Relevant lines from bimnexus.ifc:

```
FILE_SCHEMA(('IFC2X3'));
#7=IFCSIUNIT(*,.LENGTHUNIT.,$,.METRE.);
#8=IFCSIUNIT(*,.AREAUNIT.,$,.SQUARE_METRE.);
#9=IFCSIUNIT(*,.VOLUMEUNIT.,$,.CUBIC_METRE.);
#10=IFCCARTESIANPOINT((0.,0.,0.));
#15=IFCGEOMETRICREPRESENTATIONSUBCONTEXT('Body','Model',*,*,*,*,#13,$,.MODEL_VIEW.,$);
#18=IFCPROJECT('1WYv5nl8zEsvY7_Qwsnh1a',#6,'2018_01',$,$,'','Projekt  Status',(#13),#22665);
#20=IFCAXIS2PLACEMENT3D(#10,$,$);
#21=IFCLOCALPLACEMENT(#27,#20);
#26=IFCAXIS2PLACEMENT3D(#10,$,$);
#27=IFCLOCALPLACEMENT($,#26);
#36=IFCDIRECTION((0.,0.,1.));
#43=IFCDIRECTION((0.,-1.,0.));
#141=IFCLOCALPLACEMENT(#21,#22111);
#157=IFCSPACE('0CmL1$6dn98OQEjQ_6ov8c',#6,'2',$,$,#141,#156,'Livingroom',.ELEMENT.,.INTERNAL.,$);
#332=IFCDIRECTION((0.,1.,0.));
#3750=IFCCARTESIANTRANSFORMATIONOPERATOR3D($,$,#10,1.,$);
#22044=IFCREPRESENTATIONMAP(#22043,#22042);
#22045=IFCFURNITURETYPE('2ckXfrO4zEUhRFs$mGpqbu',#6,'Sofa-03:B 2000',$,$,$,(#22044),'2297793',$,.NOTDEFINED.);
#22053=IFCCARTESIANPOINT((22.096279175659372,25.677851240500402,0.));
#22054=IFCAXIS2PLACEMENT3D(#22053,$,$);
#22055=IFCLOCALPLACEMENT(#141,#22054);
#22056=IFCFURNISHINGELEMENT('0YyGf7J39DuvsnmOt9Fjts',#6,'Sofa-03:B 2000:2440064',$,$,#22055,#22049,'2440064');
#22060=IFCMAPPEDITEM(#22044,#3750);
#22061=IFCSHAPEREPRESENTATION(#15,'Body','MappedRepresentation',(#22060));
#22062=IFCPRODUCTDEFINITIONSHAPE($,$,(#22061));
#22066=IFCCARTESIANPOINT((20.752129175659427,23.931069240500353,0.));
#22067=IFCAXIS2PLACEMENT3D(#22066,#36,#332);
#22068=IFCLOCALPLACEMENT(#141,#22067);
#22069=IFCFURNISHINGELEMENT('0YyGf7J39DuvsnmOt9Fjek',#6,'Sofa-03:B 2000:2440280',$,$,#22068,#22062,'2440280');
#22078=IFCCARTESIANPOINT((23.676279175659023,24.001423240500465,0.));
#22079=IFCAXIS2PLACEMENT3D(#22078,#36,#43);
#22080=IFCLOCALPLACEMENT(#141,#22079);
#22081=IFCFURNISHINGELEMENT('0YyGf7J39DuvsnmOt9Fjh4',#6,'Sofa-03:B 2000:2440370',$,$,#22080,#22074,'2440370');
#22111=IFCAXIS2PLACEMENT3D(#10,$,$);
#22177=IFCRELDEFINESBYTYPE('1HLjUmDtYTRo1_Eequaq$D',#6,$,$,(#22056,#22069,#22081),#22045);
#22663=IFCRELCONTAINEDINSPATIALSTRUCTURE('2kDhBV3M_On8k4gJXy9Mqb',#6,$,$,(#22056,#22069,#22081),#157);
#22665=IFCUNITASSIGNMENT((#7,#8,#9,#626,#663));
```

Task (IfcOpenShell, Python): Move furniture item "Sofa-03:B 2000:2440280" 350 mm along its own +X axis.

```python
import ifcopenshell
import ifcopenshell.api.geometry
import ifcopenshell.util.placement
import ifcopenshell.util.unit

model = ifcopenshell.open("bimnexus.ifc")
unit_scale = ifcopenshell.util.unit.calculate_unit_scale(model)

item = model.by_id(22069)
matrix = ifcopenshell.util.placement.get_local_placement(item.ObjectPlacement)
matrix[:3, 3] += matrix[:3, 0] * 0.35 / unit_scale
ifcopenshell.api.geometry.edit_object_placement(model, product=item, matrix=matrix, is_si=False)

print(ifcopenshell.util.placement.get_local_placement(item.ObjectPlacement).round(3) + 0.0)

model.write("bimnexus_rev.ifc")
```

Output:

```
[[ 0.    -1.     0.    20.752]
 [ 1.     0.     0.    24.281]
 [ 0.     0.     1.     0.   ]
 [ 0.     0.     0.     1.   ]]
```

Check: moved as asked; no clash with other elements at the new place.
